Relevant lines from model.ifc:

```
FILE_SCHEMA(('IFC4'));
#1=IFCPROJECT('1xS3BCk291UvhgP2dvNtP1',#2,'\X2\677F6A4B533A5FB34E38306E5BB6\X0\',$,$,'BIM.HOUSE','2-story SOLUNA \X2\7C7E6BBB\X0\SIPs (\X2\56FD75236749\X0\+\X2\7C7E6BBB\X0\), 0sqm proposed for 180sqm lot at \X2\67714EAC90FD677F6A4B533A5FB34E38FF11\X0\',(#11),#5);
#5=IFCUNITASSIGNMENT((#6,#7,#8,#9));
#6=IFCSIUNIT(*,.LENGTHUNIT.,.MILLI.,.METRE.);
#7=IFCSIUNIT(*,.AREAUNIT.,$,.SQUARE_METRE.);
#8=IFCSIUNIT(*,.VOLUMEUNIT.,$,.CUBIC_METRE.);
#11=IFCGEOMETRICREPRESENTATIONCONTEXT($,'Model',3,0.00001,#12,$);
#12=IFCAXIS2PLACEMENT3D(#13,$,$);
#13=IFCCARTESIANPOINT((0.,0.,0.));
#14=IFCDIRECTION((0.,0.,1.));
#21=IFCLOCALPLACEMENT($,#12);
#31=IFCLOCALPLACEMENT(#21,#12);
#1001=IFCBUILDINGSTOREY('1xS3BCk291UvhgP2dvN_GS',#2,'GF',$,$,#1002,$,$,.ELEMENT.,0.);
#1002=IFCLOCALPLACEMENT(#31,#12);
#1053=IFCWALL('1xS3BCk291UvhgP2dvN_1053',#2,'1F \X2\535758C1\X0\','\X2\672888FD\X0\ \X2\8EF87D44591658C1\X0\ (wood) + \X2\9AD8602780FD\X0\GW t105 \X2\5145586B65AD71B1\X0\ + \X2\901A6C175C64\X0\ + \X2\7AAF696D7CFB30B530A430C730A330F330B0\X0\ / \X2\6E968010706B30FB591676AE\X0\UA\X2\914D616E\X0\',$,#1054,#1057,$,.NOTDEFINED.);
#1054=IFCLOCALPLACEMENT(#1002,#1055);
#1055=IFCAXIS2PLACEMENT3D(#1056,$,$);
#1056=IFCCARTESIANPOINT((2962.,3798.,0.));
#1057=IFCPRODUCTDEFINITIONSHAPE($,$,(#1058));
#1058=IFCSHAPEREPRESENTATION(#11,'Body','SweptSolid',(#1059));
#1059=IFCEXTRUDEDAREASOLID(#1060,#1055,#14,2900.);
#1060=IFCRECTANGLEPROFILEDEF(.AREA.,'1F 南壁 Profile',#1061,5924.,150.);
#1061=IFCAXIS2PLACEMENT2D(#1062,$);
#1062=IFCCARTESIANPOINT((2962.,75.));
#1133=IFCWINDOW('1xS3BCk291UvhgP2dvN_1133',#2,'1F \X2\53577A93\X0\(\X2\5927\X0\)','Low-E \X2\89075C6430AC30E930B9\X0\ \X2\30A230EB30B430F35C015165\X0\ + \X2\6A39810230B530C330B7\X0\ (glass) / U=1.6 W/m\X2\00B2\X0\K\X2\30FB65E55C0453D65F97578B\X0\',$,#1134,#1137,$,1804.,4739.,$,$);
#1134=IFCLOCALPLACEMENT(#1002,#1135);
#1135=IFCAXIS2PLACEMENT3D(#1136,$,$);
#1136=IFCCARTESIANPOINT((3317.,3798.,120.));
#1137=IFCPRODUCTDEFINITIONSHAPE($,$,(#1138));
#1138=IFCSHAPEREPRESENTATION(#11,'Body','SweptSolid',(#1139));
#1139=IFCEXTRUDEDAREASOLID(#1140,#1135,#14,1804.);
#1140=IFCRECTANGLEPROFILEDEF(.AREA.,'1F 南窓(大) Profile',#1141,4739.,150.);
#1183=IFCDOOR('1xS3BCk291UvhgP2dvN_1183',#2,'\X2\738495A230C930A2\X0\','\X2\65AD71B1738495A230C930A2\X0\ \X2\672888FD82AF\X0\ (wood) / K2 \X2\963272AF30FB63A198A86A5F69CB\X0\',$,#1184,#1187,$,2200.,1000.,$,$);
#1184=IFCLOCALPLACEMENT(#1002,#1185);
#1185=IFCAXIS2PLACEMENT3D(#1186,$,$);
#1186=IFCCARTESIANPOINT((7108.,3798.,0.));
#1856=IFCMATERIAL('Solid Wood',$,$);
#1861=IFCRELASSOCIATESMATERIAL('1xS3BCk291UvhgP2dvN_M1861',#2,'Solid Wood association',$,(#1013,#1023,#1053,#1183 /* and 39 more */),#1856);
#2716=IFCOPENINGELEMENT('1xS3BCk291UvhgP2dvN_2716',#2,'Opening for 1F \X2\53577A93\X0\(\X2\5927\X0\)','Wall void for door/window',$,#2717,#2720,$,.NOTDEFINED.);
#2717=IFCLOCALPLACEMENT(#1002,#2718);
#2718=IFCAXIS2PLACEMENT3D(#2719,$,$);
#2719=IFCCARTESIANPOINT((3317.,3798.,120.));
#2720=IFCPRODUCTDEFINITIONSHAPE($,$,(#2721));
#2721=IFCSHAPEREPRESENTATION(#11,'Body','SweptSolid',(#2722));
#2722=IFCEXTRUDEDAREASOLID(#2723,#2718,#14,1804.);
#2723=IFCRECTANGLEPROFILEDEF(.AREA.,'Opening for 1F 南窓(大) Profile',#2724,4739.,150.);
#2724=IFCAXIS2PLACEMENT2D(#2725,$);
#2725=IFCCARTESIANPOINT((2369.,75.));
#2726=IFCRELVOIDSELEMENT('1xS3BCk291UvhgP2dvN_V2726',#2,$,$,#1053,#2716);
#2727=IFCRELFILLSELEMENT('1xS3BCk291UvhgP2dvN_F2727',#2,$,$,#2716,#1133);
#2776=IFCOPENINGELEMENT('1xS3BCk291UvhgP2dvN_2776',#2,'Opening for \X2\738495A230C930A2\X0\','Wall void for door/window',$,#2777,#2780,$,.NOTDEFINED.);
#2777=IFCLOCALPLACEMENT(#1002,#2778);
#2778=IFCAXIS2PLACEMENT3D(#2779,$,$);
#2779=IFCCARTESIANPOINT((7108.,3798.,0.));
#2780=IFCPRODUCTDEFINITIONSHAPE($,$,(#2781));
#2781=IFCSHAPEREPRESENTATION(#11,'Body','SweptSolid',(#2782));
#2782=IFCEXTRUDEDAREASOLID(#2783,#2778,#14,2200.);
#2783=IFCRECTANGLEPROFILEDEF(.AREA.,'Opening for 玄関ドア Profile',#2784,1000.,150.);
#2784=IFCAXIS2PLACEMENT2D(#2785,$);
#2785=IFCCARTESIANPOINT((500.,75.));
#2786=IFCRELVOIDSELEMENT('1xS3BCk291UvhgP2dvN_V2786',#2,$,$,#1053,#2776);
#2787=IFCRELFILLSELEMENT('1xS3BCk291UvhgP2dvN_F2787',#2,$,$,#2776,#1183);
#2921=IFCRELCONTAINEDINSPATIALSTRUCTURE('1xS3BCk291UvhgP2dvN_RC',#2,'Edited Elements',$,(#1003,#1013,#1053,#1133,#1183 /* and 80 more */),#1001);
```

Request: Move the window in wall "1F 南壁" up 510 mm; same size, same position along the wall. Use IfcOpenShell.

```python
import numpy as np
import ifcopenshell
import ifcopenshell.api.geometry
import ifcopenshell.util.placement
import ifcopenshell.util.unit

model = ifcopenshell.open("model.ifc")
unit_scale = ifcopenshell.util.unit.calculate_unit_scale(model)

window = model.by_guid("1xS3BCk291UvhgP2dvN_1133")
opening = window.FillsVoids[0].RelatingOpeningElement
dz = 510.0

shift = np.array([0.0, 0.0, dz])
# The window is not placed relative to its opening, so move both.
for product in (opening, window):
    matrix = ifcopenshell.util.placement.get_local_placement(product.ObjectPlacement)
    matrix[:3, 3] += shift
    ifcopenshell.api.geometry.edit_object_placement(model, product=product, matrix=matrix, is_si=False)

print(f"moved by {dz * unit_scale:+.3f} m")

model.write("model_v2.ifc")
```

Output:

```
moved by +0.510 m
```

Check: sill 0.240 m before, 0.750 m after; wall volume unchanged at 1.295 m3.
